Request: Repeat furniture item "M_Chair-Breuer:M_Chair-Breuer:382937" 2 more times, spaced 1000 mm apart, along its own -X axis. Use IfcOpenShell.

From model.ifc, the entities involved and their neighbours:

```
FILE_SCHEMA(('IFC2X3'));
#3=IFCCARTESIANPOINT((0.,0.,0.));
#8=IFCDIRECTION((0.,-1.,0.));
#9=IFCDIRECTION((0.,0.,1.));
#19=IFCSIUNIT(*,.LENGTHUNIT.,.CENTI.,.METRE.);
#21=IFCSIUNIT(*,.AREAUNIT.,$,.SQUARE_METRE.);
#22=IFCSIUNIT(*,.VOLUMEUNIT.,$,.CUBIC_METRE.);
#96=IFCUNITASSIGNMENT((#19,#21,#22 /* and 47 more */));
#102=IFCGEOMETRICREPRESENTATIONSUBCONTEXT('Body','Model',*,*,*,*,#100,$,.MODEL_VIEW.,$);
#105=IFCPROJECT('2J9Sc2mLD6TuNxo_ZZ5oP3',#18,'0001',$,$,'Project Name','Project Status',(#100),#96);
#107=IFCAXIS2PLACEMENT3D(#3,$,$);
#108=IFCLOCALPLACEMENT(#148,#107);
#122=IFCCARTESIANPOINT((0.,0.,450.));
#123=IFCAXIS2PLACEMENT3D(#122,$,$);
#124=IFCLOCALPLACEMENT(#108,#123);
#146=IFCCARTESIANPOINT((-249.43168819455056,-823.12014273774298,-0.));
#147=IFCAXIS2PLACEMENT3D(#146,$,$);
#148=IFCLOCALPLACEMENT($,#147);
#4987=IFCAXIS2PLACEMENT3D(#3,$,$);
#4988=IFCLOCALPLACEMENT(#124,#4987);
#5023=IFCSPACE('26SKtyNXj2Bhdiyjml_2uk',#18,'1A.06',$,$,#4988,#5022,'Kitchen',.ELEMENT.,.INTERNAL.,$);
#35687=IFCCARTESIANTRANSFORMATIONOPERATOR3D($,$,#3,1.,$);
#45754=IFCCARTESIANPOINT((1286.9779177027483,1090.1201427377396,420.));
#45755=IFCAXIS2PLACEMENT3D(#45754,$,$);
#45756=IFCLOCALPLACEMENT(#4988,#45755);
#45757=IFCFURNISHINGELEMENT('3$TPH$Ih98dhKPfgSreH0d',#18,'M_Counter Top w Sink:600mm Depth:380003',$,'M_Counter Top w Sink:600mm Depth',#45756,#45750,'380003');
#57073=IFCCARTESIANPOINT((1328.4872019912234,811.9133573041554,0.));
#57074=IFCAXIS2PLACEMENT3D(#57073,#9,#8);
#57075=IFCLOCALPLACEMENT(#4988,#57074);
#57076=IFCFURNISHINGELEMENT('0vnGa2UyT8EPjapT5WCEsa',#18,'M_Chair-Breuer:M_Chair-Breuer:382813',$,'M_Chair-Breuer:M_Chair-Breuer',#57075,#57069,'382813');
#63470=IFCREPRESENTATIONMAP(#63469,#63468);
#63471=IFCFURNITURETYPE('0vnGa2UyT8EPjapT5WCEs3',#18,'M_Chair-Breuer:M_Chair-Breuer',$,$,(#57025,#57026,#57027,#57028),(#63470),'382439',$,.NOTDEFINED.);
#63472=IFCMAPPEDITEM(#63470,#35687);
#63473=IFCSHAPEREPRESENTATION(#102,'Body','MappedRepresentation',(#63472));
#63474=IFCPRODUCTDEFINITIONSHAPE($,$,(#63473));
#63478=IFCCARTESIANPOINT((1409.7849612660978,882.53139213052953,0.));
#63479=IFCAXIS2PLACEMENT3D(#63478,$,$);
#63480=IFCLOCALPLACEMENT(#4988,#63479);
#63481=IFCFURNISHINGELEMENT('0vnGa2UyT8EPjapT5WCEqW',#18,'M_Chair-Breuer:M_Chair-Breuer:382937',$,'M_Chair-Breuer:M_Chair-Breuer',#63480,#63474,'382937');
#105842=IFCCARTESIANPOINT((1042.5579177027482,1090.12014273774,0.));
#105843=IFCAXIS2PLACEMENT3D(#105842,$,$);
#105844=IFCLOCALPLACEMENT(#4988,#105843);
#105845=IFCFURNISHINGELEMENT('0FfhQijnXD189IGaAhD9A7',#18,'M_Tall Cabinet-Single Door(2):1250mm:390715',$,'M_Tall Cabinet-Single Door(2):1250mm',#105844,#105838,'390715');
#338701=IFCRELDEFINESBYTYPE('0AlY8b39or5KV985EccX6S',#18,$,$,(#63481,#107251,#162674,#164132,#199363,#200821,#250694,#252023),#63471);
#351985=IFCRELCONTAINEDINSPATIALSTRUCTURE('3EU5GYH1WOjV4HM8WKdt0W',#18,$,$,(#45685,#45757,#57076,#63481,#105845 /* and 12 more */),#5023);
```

```python
import ifcopenshell
import ifcopenshell.api.geometry
import ifcopenshell.api.root
import ifcopenshell.util.element
import ifcopenshell.util.placement
import ifcopenshell.util.unit

model = ifcopenshell.open("model.ifc")
unit_scale = ifcopenshell.util.unit.calculate_unit_scale(model)


def reuse_history(source, copy):
    """copy_class also copies each property set's owner history, people and application; keep the originals."""
    for rel in copy.IsDefinedBy:
        if rel.is_a("IfcRelDefinesByProperties") and (history := rel.RelatingPropertyDefinition.OwnerHistory):
            rel.RelatingPropertyDefinition.OwnerHistory = source.OwnerHistory
            ifcopenshell.util.element.remove_deep2(model, history)


source = model.by_guid("0vnGa2UyT8EPjapT5WCEqW")
base = ifcopenshell.util.placement.get_local_placement(source.ObjectPlacement)
step = -base[:3, 0] * 1 / unit_scale

for i in range(1, 3):
    copy = ifcopenshell.api.root.copy_class(model, product=source)
    copy.Representation = ifcopenshell.util.element.copy_deep(
        model, source.Representation, exclude=["IfcGeometricRepresentationContext", "IfcRepresentationMap"]
    )
    copy.Name = "M_Chair-Breuer:M_Chair-Breuer"
    copy.Tag = None
    reuse_history(source, copy)
    matrix = base.copy()
    matrix[:3, 3] += i * step
    print("added at", matrix[:3, 3].round(3) + 0.0)
    ifcopenshell.api.geometry.edit_object_placement(model, product=copy, matrix=matrix, is_si=False)

model.write("model_rev.ifc")
```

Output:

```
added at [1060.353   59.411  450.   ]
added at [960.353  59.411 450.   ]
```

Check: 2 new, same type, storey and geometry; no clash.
